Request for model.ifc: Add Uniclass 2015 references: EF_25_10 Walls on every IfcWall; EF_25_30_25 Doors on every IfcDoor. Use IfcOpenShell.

First a look at what the model holds.

```python
import ifcopenshell

model = ifcopenshell.open("model.ifc")
print(model.schema)
print("classifications:", [c.Name for c in model.by_type("IfcClassification")])
for ifc_class in ("IfcDoor", "IfcRoof", "IfcStair", "IfcWall", "IfcWindow"):
    print(ifc_class, len(model.by_type(ifc_class)))
```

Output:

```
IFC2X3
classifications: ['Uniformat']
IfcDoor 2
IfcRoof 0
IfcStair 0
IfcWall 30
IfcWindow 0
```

```python
import ifcopenshell
import ifcopenshell.api.classification

model = ifcopenshell.open("model.ifc")

# IFC2X3 requires Source and Edition and has no link from the project to the system.
system = model.create_entity("IfcClassification", Source="NBS", Edition="2015", Name="Uniclass 2015")

codes = {
    "IfcWall": ("EF_25_10", "Walls"),
    "IfcDoor": ("EF_25_30_25", "Doors"),
}
for ifc_class, (code, name) in codes.items():
    products = model.by_type(ifc_class)
    ifcopenshell.api.classification.add_reference(
        model, products=products, classification=system, identification=code, name=name
    )
    print(code, len(products))

model.write("model_v2.ifc")
```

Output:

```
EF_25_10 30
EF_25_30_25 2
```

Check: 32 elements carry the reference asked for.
